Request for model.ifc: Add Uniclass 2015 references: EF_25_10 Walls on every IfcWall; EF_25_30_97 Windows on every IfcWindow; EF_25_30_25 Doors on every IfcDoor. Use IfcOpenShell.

First a look at what the model holds.

```python
import ifcopenshell

model = ifcopenshell.open("model.ifc")
print(model.schema)
print("classifications:", [c.Name for c in model.by_type("IfcClassification")])
for ifc_class in ("IfcDoor", "IfcRoof", "IfcStair", "IfcWall", "IfcWindow"):
    print(ifc_class, len(model.by_type(ifc_class)))
```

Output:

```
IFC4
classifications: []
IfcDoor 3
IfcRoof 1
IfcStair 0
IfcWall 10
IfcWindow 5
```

```python
import ifcopenshell
import ifcopenshell.api.classification

model = ifcopenshell.open("model.ifc")

system = ifcopenshell.api.classification.add_classification(model, classification="Uniclass 2015")

codes = {
    "IfcWall": ("EF_25_10", "Walls"),
    "IfcWindow": ("EF_25_30_97", "Windows"),
    "IfcDoor": ("EF_25_30_25", "Doors"),
}
for ifc_class, (code, name) in codes.items():
    products = model.by_type(ifc_class)
    ifcopenshell.api.classification.add_reference(
        model, products=products, classification=system, identification=code, name=name
    )
    print(code, len(products))

model.write("model_rev.ifc")
```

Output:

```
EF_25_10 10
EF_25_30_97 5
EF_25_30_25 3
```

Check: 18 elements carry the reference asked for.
